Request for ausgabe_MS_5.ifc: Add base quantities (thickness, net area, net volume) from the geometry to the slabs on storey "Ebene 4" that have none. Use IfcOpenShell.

First a look at what the model holds.

```python
import ifcopenshell
import ifcopenshell.util.element
import ifcopenshell.util.unit

model = ifcopenshell.open("ausgabe_MS_5.ifc")
print(model.schema)
for unit_type in ("LENGTHUNIT", "AREAUNIT", "VOLUMEUNIT"):
    print(unit_type, ifcopenshell.util.unit.calculate_unit_scale(model, unit_type))
storey = next(s for s in model.by_type("IfcBuildingStorey") if s.Name == "Ebene 4")
slabs = [e for e in ifcopenshell.util.element.get_decomposition(storey) if e.is_a("IfcSlab")]
for e in sorted(slabs, key=lambda e: e.id()):
    print(e.id(), e.is_a(), e.Name, list(ifcopenshell.util.element.get_psets(e, qtos_only=True)), sep=" | ")
```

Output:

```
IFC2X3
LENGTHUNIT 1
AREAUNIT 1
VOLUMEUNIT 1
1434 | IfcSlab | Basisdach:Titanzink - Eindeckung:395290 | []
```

```python
import ifcopenshell
import ifcopenshell.api.pset
import ifcopenshell.geom
import ifcopenshell.util.element
import ifcopenshell.util.shape
import ifcopenshell.util.unit

model = ifcopenshell.open("ausgabe_MS_5.ifc")
unit_scale = ifcopenshell.util.unit.calculate_unit_scale(model)
area_scale = ifcopenshell.util.unit.calculate_unit_scale(model, "AREAUNIT")
volume_scale = ifcopenshell.util.unit.calculate_unit_scale(model, "VOLUMEUNIT")
settings = ifcopenshell.geom.settings()

storey = next(s for s in model.by_type("IfcBuildingStorey") if s.Name == "Ebene 4")
slabs = [e for e in ifcopenshell.util.element.get_decomposition(storey) if e.is_a("IfcSlab")]

for e in sorted(slabs, key=lambda e: e.id()):
    if ifcopenshell.util.element.get_psets(e, qtos_only=True, should_inherit=False):
        continue
    # Geometry comes back in metres, in the element's own axes.
    shape = ifcopenshell.geom.create_shape(settings, e)
    values = {
        "Width": ifcopenshell.util.shape.get_z(shape.geometry) / unit_scale,
        "NetArea": ifcopenshell.util.shape.get_footprint_area(shape.geometry) / area_scale,
        "NetVolume": ifcopenshell.util.shape.get_volume(shape.geometry) / volume_scale,
    }
    qto = ifcopenshell.api.pset.add_qto(model, product=e, name="BaseQuantities")
    ifcopenshell.api.pset.edit_qto(model, qto=qto, properties=values)
    print(e.id(), {k: round(v, 3) for k, v in values.items()})

model.write("ausgabe_MS_5_rev.ifc")
```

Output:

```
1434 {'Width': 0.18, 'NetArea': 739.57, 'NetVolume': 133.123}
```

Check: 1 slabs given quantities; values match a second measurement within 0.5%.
